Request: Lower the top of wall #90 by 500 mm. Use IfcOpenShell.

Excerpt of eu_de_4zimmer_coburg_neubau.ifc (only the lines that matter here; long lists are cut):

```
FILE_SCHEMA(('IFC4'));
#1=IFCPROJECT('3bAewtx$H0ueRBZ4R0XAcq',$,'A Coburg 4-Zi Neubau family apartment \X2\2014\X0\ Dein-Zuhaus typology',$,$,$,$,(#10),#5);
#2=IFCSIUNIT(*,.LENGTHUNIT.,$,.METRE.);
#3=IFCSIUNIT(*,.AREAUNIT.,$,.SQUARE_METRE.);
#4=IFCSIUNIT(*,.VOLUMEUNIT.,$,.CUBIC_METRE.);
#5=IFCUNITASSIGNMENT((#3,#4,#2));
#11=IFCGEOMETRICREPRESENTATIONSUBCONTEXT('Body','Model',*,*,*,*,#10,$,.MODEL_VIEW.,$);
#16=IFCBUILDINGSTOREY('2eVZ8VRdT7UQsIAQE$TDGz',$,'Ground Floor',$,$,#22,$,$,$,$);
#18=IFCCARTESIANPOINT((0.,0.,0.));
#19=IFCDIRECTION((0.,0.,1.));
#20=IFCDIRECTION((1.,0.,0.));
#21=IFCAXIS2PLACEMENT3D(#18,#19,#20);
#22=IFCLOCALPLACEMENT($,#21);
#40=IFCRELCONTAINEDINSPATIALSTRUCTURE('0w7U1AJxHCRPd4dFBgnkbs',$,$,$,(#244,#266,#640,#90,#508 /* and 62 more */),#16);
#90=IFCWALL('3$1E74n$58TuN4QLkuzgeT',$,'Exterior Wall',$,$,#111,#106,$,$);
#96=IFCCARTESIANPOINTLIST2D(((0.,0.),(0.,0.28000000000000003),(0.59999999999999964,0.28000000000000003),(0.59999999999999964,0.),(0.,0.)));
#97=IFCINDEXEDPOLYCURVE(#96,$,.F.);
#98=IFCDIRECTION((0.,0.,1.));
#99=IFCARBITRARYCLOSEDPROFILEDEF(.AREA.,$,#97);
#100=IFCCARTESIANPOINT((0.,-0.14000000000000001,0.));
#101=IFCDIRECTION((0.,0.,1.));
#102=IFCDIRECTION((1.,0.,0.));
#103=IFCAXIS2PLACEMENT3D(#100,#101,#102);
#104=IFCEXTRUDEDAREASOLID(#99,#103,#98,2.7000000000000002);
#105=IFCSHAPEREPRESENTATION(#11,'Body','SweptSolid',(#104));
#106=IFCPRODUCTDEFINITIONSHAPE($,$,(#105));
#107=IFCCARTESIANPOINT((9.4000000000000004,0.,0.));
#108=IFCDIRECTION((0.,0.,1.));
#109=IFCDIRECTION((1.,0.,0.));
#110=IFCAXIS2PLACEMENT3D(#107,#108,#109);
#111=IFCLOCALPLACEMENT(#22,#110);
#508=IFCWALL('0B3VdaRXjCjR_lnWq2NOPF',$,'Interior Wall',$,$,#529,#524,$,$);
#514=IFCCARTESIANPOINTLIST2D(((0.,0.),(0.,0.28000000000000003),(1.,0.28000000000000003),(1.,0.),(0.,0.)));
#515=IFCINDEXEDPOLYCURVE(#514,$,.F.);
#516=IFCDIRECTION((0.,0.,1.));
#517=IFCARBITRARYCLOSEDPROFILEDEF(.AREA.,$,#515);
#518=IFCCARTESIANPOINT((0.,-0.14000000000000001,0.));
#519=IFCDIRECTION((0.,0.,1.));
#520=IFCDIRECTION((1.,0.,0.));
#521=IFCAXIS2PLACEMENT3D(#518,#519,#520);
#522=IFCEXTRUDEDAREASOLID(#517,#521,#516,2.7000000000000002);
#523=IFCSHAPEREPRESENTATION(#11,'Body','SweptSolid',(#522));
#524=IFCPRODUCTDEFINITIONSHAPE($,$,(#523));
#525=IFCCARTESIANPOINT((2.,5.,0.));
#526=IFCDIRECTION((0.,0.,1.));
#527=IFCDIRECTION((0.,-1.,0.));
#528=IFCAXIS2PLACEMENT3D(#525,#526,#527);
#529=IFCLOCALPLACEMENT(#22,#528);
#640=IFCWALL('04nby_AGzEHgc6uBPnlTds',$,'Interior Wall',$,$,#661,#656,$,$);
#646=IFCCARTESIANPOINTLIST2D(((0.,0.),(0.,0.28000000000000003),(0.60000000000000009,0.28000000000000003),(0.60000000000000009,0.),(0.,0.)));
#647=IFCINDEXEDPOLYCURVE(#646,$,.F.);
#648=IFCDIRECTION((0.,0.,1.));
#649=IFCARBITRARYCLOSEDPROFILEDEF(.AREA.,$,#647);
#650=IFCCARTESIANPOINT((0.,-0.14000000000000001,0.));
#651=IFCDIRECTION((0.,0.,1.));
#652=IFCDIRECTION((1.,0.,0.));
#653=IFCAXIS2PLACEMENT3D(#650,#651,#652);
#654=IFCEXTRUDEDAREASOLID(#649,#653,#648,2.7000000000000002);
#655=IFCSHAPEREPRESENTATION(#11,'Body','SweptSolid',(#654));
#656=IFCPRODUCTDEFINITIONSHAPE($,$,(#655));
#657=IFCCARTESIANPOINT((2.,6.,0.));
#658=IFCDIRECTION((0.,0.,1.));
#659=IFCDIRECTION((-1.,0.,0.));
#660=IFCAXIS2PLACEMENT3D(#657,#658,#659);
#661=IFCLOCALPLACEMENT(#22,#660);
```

```python
import ifcopenshell
import ifcopenshell.geom
import ifcopenshell.util.representation
import ifcopenshell.util.shape

model = ifcopenshell.open("eu_de_4zimmer_coburg_neubau.ifc")
settings = ifcopenshell.geom.settings()


def volume(element):
    """Net volume in cubic metres, openings subtracted."""
    shape = ifcopenshell.geom.create_shape(settings, element)
    return ifcopenshell.util.shape.get_volume(shape.geometry)


wall = model.by_id(90)
before = volume(wall)

body = ifcopenshell.util.representation.get_representation(wall, "Model", "Body")
solid = body.Items[0]
old_height = solid.Depth
solid.Depth -= 0.5
after = volume(wall)

print(f"height {old_height:g} -> {solid.Depth:g}, volume {before:.3f} -> {after:.3f} m3")

model.write("eu_de_4zimmer_coburg_neubau_edited.ifc")
```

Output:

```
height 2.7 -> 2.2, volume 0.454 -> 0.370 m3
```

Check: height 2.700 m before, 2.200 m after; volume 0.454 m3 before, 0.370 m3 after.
